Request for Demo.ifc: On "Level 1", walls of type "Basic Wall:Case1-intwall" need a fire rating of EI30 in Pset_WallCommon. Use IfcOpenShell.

First a look at what the model holds.

```python
import ifcopenshell
import ifcopenshell.util.element

model = ifcopenshell.open("Demo.ifc")
print(model.schema)
storey = next(s for s in model.by_type("IfcBuildingStorey") if s.Name == "Level 1")
walls = [e for e in ifcopenshell.util.element.get_decomposition(storey) if e.is_a("IfcWall")]
seen = {}
for e in walls:
    element_type = ifcopenshell.util.element.get_type(e)
    key = (element_type.Name if element_type != e and element_type else None, ifcopenshell.util.element.get_pset(e, "Pset_WallCommon", "FireRating"))
    seen[key] = seen.get(key, 0) + 1
for (name, value), count in sorted(seen.items(), key=str):
    print(count, "x", name, "|", value)
```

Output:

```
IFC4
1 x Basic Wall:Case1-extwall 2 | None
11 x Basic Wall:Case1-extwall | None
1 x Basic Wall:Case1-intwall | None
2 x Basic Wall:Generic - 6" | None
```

```python
import ifcopenshell
import ifcopenshell.api.pset
import ifcopenshell.util.element

model = ifcopenshell.open("Demo.ifc")

storey = next(s for s in model.by_type("IfcBuildingStorey") if s.Name == "Level 1")
walls = [e for e in ifcopenshell.util.element.get_decomposition(storey) if e.is_a("IfcWall")]

count = 0
for e in walls:
    element_type = ifcopenshell.util.element.get_type(e)
    if element_type in (None, e) or element_type.Name != "Basic Wall:Case1-intwall":
        continue
    # add_pset returns the element's existing set when there is one.
    pset = ifcopenshell.api.pset.add_pset(model, product=e, name="Pset_WallCommon")
    ifcopenshell.api.pset.edit_pset(model, pset=pset, properties={"FireRating": "EI30"})
    count += 1

print(count, "walls updated")

model.write("Demo_rev.ifc")
```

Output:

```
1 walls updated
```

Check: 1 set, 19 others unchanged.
